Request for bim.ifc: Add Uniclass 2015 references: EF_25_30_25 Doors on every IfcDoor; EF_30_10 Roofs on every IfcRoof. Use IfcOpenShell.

First a look at what the model holds.

```python
import ifcopenshell

model = ifcopenshell.open("bim.ifc")
print(model.schema)
print("classifications:", [c.Name for c in model.by_type("IfcClassification")])
for ifc_class in ("IfcDoor", "IfcRoof", "IfcStair", "IfcWall", "IfcWindow"):
    print(ifc_class, len(model.by_type(ifc_class)))
```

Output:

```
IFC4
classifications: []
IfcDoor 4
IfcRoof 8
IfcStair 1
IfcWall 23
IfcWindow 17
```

```python
import ifcopenshell
import ifcopenshell.api.classification

model = ifcopenshell.open("bim.ifc")

system = ifcopenshell.api.classification.add_classification(model, classification="Uniclass 2015")

codes = {
    "IfcDoor": ("EF_25_30_25", "Doors"),
    "IfcRoof": ("EF_30_10", "Roofs"),
}
for ifc_class, (code, name) in codes.items():
    products = model.by_type(ifc_class)
    ifcopenshell.api.classification.add_reference(
        model, products=products, classification=system, identification=code, name=name
    )
    print(code, len(products))

model.write("bim_rev.ifc")
```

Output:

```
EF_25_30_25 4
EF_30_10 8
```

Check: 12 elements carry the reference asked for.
